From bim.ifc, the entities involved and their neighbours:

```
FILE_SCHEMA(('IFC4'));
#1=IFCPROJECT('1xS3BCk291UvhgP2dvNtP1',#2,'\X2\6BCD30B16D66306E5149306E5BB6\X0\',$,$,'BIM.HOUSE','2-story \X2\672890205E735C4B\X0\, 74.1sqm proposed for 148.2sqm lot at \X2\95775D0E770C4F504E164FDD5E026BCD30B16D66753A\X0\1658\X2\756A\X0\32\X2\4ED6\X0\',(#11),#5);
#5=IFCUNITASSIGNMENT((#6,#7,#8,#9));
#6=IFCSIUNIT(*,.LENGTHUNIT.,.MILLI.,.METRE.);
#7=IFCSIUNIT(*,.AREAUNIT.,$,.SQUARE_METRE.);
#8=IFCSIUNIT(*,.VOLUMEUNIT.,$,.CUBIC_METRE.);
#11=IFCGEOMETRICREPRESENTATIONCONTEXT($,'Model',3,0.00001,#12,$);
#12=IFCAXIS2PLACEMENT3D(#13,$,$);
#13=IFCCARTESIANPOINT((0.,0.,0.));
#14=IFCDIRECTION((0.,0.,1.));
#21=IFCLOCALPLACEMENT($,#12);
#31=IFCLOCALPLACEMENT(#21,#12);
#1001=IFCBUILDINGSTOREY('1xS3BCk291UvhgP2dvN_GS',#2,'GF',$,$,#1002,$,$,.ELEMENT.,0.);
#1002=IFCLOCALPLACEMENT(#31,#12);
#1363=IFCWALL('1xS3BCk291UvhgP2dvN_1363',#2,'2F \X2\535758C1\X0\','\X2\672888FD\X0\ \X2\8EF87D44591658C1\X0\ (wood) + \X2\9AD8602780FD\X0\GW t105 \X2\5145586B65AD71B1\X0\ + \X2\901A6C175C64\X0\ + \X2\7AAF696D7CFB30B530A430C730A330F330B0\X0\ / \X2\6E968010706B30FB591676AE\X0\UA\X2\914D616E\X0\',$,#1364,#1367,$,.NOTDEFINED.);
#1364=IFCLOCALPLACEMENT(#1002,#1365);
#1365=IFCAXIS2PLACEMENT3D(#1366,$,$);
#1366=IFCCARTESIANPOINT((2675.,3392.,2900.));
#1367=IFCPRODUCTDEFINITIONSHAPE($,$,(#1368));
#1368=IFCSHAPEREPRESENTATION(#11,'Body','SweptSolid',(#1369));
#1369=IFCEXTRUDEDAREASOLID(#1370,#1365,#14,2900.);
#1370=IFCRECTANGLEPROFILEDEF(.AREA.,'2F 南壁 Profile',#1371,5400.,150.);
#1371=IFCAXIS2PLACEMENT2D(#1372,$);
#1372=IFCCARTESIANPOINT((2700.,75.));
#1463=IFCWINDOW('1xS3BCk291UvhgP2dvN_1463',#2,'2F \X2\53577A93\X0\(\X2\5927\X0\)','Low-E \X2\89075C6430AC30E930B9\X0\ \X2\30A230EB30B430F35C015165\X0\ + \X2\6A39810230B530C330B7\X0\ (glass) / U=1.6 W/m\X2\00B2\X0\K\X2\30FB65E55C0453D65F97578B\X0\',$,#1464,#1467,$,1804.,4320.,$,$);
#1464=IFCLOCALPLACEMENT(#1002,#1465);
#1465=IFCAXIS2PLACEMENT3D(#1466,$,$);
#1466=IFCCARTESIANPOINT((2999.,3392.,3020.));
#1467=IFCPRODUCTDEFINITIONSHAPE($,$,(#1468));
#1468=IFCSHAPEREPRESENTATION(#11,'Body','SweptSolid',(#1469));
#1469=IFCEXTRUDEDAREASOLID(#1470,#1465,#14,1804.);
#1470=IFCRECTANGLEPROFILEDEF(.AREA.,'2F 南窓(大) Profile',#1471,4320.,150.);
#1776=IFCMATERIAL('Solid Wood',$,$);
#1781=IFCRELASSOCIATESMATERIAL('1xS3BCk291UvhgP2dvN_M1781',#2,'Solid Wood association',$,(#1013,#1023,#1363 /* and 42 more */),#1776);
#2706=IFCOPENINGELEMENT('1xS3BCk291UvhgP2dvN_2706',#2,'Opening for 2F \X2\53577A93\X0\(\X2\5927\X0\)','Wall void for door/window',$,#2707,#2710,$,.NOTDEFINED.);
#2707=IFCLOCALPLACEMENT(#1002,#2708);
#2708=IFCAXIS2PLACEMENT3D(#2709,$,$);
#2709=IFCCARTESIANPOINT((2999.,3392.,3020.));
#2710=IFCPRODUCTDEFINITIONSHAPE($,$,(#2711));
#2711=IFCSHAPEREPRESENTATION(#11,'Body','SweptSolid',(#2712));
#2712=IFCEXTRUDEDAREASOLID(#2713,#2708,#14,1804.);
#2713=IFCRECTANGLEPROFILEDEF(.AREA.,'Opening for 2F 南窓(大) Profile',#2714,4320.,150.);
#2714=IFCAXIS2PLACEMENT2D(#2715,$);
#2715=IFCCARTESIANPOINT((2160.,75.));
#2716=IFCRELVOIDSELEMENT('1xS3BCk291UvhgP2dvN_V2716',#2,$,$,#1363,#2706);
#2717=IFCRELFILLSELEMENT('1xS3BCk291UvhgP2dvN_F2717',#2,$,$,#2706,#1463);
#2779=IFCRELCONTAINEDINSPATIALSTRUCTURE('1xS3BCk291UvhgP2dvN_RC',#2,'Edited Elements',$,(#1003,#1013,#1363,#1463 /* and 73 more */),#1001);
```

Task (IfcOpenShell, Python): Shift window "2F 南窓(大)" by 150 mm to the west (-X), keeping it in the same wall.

```python
import ifcopenshell
import ifcopenshell.api.geometry
import ifcopenshell.util.placement
import ifcopenshell.util.unit

model = ifcopenshell.open("bim.ifc")
unit_scale = ifcopenshell.util.unit.calculate_unit_scale(model)

window = model.by_guid("1xS3BCk291UvhgP2dvN_1463")
opening = window.FillsVoids[0].RelatingOpeningElement
wall = opening.VoidsElements[0].RelatingBuildingElement

wall_matrix = ifcopenshell.util.placement.get_local_placement(wall.ObjectPlacement)
shift = wall_matrix[:3, 0] * -0.15 / unit_scale
before = ifcopenshell.util.placement.get_local_placement(window.ObjectPlacement)[:3, 3].copy()

# The window is not placed relative to its opening, so move both.
for product in (opening, window):
    matrix = ifcopenshell.util.placement.get_local_placement(product.ObjectPlacement)
    matrix[:3, 3] += shift
    ifcopenshell.api.geometry.edit_object_placement(model, product=product, matrix=matrix, is_si=False)

after = ifcopenshell.util.placement.get_local_placement(window.ObjectPlacement)[:3, 3]
print("window moved by", (after - before).round(3) + 0.0)

model.write("bim_rev.ifc")
```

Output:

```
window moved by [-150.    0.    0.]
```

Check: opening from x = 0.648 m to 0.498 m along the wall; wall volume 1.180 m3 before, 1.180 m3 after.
